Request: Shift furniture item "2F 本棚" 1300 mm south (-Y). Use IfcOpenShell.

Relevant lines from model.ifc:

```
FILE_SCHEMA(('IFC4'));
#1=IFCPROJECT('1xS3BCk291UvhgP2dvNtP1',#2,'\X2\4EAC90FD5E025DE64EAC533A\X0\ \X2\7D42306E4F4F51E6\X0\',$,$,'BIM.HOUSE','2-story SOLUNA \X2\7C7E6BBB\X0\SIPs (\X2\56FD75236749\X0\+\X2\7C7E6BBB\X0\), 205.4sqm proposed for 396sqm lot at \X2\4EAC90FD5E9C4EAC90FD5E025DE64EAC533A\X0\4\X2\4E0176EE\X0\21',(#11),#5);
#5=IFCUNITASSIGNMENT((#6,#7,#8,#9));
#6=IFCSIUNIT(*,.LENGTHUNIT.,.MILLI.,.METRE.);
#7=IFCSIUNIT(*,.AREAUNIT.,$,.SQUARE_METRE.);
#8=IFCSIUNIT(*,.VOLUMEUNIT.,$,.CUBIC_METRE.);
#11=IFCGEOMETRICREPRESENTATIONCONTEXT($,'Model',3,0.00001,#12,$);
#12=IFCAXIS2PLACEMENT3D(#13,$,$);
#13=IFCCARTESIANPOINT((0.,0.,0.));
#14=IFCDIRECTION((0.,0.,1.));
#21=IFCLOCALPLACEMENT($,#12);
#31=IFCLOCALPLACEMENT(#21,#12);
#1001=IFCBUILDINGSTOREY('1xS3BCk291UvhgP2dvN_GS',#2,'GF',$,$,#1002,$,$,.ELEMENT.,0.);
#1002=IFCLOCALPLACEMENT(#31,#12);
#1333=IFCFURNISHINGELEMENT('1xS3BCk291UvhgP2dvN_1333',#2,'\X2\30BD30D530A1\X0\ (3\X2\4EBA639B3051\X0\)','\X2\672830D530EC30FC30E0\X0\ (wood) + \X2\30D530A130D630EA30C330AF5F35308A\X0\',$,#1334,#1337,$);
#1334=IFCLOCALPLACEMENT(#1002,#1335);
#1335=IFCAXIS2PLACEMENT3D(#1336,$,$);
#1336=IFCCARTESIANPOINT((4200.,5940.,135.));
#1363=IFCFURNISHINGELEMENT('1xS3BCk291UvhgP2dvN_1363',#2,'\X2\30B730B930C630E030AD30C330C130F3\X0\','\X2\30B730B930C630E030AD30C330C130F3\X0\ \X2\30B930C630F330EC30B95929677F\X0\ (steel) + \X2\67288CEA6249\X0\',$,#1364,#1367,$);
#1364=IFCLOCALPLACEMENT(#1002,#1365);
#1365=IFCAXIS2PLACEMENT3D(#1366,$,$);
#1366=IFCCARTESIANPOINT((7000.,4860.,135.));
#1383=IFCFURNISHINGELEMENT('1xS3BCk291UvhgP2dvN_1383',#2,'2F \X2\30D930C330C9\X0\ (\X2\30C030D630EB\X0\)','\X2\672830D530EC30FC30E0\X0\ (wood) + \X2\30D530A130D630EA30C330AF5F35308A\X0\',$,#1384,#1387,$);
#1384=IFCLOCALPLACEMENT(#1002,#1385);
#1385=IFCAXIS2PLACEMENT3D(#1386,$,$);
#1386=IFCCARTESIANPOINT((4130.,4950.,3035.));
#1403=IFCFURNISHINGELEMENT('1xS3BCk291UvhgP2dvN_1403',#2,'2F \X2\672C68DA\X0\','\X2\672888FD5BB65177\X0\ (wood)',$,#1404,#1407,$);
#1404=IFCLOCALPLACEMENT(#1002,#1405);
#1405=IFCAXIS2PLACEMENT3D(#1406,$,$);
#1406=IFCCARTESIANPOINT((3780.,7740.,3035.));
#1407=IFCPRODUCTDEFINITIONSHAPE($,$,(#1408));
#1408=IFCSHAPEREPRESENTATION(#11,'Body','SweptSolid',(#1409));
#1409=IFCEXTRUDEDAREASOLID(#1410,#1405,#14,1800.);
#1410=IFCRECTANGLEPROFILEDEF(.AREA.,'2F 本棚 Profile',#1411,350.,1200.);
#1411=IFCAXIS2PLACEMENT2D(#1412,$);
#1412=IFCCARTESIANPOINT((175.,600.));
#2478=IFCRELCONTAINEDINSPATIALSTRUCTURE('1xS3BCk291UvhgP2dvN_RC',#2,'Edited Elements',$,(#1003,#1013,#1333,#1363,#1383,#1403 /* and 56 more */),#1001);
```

```python
import ifcopenshell
import ifcopenshell.api.geometry
import ifcopenshell.util.placement
import ifcopenshell.util.unit

model = ifcopenshell.open("model.ifc")
unit_scale = ifcopenshell.util.unit.calculate_unit_scale(model)

item = model.by_guid("1xS3BCk291UvhgP2dvN_1403")
matrix = ifcopenshell.util.placement.get_local_placement(item.ObjectPlacement)
matrix[1, 3] -= 1.3 / unit_scale
ifcopenshell.api.geometry.edit_object_placement(model, product=item, matrix=matrix, is_si=False)

print(ifcopenshell.util.placement.get_local_placement(item.ObjectPlacement).round(3) + 0.0)

model.write("model_rev.ifc")
```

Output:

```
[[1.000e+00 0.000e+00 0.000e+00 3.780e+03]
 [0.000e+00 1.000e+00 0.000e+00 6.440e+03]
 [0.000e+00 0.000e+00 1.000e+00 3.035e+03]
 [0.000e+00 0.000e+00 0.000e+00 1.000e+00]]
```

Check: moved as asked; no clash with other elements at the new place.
